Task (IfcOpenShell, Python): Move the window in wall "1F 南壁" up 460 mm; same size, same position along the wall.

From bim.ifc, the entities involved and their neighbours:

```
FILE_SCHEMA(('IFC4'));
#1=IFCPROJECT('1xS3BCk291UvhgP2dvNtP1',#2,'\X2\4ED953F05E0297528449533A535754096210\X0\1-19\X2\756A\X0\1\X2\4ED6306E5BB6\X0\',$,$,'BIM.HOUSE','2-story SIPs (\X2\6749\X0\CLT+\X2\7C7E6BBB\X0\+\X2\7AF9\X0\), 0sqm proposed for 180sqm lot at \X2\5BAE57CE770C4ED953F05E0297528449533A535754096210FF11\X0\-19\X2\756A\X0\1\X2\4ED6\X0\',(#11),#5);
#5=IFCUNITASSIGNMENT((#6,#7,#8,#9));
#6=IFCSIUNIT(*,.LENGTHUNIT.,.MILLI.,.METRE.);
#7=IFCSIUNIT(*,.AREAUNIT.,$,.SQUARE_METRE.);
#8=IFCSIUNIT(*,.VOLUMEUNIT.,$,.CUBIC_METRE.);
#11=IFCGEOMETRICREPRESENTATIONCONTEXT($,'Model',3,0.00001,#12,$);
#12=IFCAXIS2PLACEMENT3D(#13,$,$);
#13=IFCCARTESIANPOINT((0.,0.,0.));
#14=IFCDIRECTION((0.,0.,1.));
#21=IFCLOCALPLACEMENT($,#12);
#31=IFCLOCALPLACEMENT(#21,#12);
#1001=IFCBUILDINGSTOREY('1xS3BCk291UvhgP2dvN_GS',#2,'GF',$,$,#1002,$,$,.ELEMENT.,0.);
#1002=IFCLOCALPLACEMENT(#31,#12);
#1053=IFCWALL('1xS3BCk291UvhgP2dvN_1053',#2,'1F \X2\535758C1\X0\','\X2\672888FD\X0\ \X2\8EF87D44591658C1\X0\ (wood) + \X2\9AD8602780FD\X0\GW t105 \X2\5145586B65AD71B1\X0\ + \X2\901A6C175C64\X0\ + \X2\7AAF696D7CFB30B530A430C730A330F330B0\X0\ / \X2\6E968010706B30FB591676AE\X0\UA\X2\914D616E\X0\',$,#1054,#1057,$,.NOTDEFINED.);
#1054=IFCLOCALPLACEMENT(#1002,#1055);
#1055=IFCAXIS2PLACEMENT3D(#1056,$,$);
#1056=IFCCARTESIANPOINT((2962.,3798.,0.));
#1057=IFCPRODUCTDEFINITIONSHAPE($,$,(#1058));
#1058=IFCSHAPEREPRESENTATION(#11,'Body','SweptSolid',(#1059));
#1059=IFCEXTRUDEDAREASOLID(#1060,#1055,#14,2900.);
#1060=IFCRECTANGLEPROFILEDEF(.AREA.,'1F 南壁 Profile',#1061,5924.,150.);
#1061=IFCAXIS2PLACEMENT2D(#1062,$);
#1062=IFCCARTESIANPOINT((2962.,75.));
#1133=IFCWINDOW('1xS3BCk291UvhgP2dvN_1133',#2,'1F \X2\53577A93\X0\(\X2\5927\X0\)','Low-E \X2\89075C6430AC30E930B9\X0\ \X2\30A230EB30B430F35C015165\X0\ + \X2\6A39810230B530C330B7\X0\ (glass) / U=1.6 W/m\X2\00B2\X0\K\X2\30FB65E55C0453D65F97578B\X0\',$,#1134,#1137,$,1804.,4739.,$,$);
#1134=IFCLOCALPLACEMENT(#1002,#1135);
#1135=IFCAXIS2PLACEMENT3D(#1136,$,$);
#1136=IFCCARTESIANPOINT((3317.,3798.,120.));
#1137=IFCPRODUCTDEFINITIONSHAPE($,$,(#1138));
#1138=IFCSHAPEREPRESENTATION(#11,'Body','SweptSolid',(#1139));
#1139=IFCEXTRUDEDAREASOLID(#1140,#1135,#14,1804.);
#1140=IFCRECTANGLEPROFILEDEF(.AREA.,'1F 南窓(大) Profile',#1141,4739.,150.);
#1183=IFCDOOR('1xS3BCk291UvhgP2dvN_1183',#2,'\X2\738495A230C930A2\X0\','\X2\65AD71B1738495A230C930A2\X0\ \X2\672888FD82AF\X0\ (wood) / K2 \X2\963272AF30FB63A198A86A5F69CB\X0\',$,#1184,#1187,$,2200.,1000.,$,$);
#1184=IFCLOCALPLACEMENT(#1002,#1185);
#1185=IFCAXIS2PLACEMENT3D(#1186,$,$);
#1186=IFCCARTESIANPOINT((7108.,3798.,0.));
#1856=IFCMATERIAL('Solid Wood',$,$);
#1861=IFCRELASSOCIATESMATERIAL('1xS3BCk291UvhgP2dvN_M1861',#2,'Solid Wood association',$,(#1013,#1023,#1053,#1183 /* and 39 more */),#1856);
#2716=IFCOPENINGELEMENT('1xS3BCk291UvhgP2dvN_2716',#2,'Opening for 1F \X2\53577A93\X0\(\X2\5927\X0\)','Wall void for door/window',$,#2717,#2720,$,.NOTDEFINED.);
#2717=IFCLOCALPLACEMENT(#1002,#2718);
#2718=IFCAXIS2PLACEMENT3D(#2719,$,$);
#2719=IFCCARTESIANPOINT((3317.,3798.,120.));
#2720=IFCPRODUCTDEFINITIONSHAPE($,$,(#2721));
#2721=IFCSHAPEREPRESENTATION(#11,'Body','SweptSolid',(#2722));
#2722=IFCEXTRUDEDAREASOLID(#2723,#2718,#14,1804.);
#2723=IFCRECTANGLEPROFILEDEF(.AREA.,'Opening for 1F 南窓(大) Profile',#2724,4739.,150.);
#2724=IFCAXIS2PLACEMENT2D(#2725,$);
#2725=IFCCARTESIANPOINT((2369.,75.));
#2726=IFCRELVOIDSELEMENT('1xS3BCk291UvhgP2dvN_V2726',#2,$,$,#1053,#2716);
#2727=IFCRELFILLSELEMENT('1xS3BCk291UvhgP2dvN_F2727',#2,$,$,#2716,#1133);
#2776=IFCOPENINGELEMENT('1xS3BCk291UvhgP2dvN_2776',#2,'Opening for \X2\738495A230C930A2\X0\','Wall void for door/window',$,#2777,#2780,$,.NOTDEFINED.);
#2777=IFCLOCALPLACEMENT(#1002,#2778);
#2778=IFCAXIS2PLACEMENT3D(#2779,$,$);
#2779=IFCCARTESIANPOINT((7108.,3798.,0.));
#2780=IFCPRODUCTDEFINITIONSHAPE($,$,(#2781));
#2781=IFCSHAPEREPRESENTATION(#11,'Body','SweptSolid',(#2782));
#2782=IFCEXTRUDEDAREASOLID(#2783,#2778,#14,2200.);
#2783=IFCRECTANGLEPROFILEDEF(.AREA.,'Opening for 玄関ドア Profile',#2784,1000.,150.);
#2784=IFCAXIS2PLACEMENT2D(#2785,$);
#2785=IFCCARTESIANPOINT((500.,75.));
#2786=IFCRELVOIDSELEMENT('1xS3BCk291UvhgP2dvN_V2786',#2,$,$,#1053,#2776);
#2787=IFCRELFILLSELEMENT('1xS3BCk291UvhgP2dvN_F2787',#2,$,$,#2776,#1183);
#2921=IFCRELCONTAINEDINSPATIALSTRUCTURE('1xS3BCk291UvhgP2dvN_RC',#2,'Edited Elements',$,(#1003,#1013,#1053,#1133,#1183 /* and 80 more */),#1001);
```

```python
import numpy as np
import ifcopenshell
import ifcopenshell.api.geometry
import ifcopenshell.util.placement
import ifcopenshell.util.unit

model = ifcopenshell.open("bim.ifc")
unit_scale = ifcopenshell.util.unit.calculate_unit_scale(model)

window = model.by_guid("1xS3BCk291UvhgP2dvN_1133")
opening = window.FillsVoids[0].RelatingOpeningElement
dz = 460.0

shift = np.array([0.0, 0.0, dz])
# The window is not placed relative to its opening, so move both.
for product in (opening, window):
    matrix = ifcopenshell.util.placement.get_local_placement(product.ObjectPlacement)
    matrix[:3, 3] += shift
    ifcopenshell.api.geometry.edit_object_placement(model, product=product, matrix=matrix, is_si=False)

print(f"moved by {dz * unit_scale:+.3f} m")

model.write("bim_updated.ifc")
```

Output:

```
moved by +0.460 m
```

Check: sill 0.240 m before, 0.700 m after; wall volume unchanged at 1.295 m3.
